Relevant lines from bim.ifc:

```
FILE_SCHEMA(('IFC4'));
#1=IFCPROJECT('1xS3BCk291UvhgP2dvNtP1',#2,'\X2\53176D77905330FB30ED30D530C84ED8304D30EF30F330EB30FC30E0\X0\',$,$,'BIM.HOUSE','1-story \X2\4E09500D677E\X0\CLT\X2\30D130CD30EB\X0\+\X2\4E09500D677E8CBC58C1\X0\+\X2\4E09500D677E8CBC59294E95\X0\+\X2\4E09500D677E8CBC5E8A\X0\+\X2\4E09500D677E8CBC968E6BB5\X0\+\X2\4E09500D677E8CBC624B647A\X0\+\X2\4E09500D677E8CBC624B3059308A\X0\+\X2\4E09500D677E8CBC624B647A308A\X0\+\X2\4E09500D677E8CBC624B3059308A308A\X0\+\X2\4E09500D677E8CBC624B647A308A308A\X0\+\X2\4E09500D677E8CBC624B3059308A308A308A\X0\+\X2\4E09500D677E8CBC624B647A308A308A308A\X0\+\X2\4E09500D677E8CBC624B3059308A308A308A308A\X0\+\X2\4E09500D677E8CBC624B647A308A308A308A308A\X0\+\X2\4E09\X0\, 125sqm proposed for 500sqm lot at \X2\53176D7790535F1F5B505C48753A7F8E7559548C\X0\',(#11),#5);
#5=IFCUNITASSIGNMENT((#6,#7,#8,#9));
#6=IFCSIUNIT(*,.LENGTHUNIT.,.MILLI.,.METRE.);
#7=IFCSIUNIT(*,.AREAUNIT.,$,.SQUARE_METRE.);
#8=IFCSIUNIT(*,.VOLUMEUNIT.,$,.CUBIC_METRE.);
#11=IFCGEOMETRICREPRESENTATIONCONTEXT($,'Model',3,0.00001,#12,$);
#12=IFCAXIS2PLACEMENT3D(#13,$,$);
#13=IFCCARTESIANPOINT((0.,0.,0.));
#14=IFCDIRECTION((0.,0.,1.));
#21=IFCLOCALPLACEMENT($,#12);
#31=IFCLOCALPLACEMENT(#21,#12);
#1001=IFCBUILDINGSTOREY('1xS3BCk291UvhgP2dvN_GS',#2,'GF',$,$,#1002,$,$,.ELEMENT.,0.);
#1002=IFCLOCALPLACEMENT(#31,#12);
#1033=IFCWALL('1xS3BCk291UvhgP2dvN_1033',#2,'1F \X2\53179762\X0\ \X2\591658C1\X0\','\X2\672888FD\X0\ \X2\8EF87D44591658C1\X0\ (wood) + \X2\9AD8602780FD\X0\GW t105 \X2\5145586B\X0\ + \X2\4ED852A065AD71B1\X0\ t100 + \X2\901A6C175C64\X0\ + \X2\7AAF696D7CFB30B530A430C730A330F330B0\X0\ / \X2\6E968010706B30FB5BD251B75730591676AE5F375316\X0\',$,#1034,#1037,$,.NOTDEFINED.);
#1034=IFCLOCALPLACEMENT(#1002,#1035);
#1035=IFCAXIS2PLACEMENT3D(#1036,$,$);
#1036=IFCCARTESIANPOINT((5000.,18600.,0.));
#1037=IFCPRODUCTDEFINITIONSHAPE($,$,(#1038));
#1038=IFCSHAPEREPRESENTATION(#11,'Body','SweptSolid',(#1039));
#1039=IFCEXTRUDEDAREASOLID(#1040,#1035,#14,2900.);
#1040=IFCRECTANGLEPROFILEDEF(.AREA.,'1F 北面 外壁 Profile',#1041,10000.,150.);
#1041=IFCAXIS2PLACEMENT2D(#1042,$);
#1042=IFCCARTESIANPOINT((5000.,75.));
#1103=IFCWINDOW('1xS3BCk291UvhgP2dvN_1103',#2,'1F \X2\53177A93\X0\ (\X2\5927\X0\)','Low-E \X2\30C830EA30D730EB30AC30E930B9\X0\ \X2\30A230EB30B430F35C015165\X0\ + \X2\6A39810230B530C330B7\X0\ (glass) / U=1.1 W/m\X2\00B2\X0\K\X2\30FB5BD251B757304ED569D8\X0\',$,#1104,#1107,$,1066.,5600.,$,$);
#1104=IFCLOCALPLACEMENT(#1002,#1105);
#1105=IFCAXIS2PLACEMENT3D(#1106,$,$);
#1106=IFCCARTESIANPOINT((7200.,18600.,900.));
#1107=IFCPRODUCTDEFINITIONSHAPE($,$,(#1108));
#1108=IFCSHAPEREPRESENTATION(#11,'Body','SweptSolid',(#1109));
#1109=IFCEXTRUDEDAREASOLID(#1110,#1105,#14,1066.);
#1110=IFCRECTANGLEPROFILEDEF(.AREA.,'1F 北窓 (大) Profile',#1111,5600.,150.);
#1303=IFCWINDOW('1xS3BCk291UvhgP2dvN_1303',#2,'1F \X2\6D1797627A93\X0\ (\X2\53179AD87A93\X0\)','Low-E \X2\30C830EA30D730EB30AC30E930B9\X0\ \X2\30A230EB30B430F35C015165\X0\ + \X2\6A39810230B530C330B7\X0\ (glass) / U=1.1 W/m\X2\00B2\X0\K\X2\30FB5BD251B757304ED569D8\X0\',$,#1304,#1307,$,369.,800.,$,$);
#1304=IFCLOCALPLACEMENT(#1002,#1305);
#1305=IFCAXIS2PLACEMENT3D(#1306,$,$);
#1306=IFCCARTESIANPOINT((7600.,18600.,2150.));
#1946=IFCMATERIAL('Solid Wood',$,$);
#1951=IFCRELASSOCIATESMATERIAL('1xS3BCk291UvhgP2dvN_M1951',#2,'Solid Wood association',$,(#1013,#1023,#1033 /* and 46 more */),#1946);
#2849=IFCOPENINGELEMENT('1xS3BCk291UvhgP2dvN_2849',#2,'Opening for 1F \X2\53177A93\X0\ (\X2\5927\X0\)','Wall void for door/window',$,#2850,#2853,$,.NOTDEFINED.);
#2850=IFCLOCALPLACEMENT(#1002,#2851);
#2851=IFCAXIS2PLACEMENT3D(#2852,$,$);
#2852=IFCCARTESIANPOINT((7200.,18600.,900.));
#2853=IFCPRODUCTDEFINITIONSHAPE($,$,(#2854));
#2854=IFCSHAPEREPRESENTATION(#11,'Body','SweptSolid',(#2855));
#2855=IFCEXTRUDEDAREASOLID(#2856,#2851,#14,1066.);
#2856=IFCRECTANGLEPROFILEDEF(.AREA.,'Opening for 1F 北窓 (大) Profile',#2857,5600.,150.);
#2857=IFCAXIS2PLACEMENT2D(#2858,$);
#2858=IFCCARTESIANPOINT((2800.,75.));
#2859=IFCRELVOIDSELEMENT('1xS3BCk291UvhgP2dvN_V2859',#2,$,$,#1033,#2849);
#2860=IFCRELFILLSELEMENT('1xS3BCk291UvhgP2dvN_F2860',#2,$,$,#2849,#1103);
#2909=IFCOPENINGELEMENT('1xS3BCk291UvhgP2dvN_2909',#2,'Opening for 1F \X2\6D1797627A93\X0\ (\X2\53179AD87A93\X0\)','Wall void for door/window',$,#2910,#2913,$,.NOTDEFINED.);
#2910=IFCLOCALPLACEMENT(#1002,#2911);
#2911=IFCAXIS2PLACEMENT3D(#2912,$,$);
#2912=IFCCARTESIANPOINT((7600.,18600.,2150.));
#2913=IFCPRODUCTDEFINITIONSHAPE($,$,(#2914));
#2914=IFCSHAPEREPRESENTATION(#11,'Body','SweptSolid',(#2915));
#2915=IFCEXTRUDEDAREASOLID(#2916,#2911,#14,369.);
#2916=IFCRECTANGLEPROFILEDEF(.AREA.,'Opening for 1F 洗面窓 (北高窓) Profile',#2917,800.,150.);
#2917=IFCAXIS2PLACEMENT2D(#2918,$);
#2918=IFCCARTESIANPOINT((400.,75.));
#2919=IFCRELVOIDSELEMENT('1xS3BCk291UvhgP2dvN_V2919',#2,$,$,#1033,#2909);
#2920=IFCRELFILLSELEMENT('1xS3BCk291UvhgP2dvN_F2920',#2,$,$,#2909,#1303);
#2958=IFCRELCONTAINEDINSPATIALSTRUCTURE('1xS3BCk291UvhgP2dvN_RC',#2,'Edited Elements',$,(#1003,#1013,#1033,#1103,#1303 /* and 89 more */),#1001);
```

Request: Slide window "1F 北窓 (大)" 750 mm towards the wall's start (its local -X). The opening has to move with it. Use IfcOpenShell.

```python
import ifcopenshell
import ifcopenshell.api.geometry
import ifcopenshell.util.placement

model = ifcopenshell.open("bim.ifc")

window = model.by_guid("1xS3BCk291UvhgP2dvN_1103")
opening = window.FillsVoids[0].RelatingOpeningElement
wall = opening.VoidsElements[0].RelatingBuildingElement

wall_matrix = ifcopenshell.util.placement.get_local_placement(wall.ObjectPlacement)
shift = wall_matrix[:3, 0] * -750.0
before = ifcopenshell.util.placement.get_local_placement(window.ObjectPlacement)[:3, 3].copy()

# The window is not placed relative to its opening, so move both.
for product in (opening, window):
    matrix = ifcopenshell.util.placement.get_local_placement(product.ObjectPlacement)
    matrix[:3, 3] += shift
    ifcopenshell.api.geometry.edit_object_placement(model, product=product, matrix=matrix, is_si=False)

after = ifcopenshell.util.placement.get_local_placement(window.ObjectPlacement)[:3, 3]
print("window moved by", (after - before).round(3) + 0.0)

model.write("bim_updated.ifc")
```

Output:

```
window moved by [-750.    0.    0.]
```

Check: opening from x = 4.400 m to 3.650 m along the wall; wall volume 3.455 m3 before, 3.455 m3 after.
